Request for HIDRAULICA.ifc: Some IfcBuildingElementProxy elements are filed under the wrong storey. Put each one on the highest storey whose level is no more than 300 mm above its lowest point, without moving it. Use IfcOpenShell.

First a look at what the model holds.

```python
import ifcopenshell
import ifcopenshell.util.element
import ifcopenshell.util.placement

model = ifcopenshell.open("HIDRAULICA.ifc")
print(model.schema)
for storey in model.by_type("IfcBuildingStorey"):
    level = ifcopenshell.util.placement.get_storey_elevation(storey)
    count = sum(e.is_a("IfcBuildingElementProxy") for e in ifcopenshell.util.element.get_contained(storey))
    print(storey.id(), storey.Name, round(level, 3), count, sep=" | ")
```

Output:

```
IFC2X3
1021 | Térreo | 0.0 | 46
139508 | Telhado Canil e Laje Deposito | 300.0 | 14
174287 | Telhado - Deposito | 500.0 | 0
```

```python
import ifcopenshell
import ifcopenshell.api.spatial
import ifcopenshell.geom
import ifcopenshell.util.element
import ifcopenshell.util.placement
import ifcopenshell.util.shape
import ifcopenshell.util.unit

model = ifcopenshell.open("HIDRAULICA.ifc")
unit_scale = ifcopenshell.util.unit.calculate_unit_scale(model)
settings = ifcopenshell.geom.settings()

levels = sorted(
    ((ifcopenshell.util.placement.get_storey_elevation(s) * unit_scale, s) for s in model.by_type("IfcBuildingStorey")),
    key=lambda pair: pair[0],
)

for e in model.by_type("IfcBuildingElementProxy"):
    current = e.ContainedInStructure[0].RelatingStructure if e.ContainedInStructure else None
    if current is None or not current.is_a("IfcBuildingStorey"):
        continue
    shape = ifcopenshell.geom.create_shape(settings, e)
    bottom = ifcopenshell.util.shape.get_shape_bottom_elevation(shape, shape.geometry)
    below = [s for level, s in levels if level <= bottom + 0.3]
    storey = below[-1] if below else levels[0][1]
    if storey != current:
        # assign_container keeps the world position.
        ifcopenshell.api.spatial.assign_container(model, products=[e], relating_structure=storey)
        print(e.id(), current.Name, "->", storey.Name)

model.write("HIDRAULICA_rev.ifc")
```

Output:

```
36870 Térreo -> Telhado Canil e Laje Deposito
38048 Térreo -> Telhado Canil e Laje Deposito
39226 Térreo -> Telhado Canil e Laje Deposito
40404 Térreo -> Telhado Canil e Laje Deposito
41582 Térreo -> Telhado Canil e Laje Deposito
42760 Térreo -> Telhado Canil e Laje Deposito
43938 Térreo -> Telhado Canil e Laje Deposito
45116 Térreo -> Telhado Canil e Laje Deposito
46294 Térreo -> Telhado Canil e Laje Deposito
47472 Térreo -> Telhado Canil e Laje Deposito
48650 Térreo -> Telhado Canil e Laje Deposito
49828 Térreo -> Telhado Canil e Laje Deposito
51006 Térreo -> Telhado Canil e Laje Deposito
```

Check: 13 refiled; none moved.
